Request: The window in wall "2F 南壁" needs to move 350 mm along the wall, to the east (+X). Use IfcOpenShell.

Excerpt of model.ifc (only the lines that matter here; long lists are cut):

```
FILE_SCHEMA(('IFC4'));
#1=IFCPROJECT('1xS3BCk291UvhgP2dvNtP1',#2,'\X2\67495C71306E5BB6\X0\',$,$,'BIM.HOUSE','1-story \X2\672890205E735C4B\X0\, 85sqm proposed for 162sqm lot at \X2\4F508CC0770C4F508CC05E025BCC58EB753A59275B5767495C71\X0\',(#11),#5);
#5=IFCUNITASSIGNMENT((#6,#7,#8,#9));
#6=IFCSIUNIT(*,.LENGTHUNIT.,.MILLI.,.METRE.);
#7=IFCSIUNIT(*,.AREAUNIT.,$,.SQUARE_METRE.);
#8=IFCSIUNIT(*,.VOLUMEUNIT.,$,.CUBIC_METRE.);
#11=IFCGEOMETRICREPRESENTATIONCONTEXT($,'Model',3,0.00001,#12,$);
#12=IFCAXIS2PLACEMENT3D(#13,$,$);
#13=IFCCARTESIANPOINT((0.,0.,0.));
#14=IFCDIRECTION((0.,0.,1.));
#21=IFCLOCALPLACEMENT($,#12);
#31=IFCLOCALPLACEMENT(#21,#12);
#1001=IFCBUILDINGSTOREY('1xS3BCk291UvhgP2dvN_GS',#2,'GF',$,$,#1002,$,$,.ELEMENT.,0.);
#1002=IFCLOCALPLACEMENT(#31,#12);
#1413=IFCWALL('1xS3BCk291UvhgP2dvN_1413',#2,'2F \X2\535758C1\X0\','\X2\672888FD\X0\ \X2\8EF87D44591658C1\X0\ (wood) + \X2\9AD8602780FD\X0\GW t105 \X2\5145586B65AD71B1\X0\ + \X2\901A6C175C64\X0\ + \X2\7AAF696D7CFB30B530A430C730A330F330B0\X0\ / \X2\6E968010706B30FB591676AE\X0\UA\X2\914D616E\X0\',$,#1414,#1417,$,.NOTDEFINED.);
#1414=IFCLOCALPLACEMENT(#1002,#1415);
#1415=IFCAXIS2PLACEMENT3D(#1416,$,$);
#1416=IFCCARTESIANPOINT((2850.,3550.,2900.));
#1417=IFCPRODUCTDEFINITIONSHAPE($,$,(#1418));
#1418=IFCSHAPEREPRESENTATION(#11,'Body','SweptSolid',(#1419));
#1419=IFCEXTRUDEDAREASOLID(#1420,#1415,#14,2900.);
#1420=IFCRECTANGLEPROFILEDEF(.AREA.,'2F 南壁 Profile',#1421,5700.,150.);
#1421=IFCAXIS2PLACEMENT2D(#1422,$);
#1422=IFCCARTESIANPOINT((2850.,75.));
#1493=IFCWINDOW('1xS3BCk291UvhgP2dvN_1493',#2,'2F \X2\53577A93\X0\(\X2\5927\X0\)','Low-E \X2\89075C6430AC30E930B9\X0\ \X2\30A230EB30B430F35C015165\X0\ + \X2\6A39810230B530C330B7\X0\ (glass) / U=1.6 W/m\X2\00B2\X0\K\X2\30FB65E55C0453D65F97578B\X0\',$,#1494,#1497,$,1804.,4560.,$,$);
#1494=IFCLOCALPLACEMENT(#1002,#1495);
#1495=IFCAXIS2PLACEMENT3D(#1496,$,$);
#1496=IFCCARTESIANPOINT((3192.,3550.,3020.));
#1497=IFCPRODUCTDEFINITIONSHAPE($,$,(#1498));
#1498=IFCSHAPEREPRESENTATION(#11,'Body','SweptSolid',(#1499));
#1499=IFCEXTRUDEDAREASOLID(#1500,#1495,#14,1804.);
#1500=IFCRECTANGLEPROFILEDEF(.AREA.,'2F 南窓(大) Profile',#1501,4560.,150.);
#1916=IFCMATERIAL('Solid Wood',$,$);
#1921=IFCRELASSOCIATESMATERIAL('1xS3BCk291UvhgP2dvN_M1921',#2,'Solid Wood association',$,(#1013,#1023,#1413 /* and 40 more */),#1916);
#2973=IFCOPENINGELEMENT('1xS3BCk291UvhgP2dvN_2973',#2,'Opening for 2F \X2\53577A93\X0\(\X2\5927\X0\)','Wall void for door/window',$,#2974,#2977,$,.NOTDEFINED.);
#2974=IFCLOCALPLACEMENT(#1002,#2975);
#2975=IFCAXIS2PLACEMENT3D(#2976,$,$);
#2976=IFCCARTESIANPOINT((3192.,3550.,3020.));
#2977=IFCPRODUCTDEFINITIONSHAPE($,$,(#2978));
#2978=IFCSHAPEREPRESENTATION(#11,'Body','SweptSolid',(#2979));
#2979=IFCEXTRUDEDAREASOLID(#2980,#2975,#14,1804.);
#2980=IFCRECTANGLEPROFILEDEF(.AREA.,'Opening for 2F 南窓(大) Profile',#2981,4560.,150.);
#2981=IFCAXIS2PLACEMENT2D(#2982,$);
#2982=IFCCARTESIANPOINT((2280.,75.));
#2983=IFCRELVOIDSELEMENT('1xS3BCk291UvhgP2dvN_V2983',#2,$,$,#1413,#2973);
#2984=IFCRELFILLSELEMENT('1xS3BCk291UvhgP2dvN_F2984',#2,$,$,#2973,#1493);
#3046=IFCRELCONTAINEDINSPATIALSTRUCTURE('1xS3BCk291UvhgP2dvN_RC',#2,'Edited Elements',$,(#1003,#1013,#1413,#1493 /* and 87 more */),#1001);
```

```python
import ifcopenshell
import ifcopenshell.api.geometry
import ifcopenshell.util.placement

model = ifcopenshell.open("model.ifc")

window = model.by_guid("1xS3BCk291UvhgP2dvN_1493")
opening = window.FillsVoids[0].RelatingOpeningElement
wall = opening.VoidsElements[0].RelatingBuildingElement

wall_matrix = ifcopenshell.util.placement.get_local_placement(wall.ObjectPlacement)
shift = wall_matrix[:3, 0] * 350.0
before = ifcopenshell.util.placement.get_local_placement(window.ObjectPlacement)[:3, 3].copy()

# The window is not placed relative to its opening, so move both.
for product in (opening, window):
    matrix = ifcopenshell.util.placement.get_local_placement(product.ObjectPlacement)
    matrix[:3, 3] += shift
    ifcopenshell.api.geometry.edit_object_placement(model, product=product, matrix=matrix, is_si=False)

after = ifcopenshell.util.placement.get_local_placement(window.ObjectPlacement)[:3, 3]
print("window moved by", (after - before).round(3) + 0.0)

model.write("model_v2.ifc")
```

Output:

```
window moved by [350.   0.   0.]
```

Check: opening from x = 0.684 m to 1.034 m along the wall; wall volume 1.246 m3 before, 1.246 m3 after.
